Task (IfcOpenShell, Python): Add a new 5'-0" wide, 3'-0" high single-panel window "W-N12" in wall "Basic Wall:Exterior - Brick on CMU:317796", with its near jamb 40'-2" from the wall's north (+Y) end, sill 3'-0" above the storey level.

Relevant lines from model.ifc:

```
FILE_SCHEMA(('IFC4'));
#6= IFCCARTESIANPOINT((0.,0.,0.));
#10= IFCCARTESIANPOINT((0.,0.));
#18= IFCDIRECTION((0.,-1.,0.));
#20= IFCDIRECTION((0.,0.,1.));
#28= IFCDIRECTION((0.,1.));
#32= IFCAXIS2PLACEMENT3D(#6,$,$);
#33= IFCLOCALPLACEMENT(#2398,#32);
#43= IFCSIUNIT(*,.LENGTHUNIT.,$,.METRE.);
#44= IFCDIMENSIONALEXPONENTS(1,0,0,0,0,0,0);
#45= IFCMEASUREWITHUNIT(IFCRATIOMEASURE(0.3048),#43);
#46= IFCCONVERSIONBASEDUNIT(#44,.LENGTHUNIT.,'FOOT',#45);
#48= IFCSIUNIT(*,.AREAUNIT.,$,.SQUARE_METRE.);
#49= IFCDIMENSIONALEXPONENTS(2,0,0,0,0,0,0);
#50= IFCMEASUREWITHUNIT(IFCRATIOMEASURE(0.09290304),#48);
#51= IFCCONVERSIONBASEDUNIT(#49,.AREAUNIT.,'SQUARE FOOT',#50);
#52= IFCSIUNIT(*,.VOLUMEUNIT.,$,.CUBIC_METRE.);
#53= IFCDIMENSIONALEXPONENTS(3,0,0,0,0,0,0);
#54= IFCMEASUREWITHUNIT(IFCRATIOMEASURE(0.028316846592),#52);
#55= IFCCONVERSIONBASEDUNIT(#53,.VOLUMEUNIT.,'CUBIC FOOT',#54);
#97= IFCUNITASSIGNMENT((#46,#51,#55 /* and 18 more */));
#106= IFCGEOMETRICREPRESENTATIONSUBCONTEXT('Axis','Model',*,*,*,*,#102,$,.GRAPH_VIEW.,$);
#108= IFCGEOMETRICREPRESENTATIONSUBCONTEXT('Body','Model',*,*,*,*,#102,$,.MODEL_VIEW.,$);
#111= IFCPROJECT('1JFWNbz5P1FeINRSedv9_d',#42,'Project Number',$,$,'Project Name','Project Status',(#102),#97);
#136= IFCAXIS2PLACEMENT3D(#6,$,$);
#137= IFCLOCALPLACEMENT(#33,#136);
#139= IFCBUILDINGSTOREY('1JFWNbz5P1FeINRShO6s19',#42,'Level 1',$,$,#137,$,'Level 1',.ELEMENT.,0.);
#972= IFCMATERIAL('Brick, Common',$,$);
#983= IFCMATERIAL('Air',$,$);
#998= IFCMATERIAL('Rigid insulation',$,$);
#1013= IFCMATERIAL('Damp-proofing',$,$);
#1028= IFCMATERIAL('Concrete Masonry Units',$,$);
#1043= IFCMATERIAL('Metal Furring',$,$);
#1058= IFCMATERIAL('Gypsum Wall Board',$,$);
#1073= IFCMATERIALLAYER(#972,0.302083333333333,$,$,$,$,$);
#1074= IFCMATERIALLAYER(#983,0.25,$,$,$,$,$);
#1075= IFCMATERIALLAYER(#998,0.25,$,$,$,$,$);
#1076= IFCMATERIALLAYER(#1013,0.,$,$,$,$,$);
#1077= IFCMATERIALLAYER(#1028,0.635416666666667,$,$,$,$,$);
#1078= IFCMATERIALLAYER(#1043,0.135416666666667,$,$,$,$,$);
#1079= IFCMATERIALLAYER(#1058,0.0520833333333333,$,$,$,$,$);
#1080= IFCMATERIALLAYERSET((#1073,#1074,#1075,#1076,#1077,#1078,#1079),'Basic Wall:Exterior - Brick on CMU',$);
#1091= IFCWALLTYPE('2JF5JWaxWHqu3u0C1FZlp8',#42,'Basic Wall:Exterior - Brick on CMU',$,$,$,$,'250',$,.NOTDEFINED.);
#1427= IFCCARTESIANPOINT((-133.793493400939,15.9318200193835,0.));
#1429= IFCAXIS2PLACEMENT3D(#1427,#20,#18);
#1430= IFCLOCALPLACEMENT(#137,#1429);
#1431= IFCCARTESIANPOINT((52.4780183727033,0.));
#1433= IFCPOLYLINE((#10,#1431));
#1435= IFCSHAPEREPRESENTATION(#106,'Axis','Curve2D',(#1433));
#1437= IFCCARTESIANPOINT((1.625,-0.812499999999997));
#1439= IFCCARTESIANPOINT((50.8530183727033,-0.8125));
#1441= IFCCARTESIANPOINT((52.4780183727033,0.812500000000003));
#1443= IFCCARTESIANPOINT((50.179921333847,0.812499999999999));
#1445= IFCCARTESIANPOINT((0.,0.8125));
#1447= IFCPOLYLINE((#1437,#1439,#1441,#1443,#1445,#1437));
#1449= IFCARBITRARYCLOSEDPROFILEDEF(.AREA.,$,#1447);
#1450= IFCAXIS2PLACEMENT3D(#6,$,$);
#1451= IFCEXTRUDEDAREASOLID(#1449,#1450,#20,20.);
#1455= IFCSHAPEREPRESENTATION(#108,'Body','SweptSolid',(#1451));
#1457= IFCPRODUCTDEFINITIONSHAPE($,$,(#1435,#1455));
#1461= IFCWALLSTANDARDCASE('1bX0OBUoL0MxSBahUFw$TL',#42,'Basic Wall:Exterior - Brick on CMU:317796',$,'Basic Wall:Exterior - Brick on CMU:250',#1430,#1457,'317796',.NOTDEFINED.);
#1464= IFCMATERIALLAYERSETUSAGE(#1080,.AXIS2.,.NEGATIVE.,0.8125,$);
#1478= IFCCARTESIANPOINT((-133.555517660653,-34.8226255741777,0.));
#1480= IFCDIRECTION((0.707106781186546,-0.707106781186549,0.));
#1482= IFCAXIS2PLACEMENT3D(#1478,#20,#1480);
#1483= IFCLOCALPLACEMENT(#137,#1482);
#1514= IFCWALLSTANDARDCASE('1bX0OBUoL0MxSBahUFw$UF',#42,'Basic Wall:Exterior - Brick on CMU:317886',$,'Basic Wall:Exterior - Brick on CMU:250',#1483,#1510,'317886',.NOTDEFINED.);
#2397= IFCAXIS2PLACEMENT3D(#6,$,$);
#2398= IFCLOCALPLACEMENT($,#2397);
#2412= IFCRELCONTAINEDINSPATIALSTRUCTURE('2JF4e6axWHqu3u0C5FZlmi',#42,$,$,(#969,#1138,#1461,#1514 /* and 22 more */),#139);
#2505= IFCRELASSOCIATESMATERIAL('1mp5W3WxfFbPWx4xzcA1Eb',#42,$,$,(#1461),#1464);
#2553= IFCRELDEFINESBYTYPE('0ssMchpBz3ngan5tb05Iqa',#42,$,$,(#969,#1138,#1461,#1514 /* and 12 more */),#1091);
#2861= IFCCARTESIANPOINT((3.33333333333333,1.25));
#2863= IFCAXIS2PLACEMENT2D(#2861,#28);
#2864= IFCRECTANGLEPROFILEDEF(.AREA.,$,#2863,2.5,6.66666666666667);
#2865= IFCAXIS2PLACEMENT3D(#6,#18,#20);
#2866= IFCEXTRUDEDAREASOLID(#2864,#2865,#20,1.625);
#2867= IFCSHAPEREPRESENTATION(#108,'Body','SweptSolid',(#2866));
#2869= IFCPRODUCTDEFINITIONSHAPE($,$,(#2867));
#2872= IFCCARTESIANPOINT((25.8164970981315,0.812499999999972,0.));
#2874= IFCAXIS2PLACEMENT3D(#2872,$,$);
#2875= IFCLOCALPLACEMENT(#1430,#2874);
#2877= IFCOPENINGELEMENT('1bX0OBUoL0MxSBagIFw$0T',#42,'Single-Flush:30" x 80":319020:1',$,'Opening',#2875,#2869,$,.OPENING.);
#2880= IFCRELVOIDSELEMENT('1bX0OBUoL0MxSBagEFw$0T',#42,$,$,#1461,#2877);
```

```python
import numpy as np
import ifcopenshell
import ifcopenshell.api.feature
import ifcopenshell.api.geometry
import ifcopenshell.api.root
import ifcopenshell.api.spatial
import ifcopenshell.geom
import ifcopenshell.util.element
import ifcopenshell.util.placement
import ifcopenshell.util.representation
import ifcopenshell.util.shape
import ifcopenshell.util.unit

model = ifcopenshell.open("model.ifc")
unit_scale = ifcopenshell.util.unit.calculate_unit_scale(model)
settings = ifcopenshell.geom.settings()


def volume(element):
    """Net volume in cubic metres, openings subtracted."""
    shape = ifcopenshell.geom.create_shape(settings, element)
    return ifcopenshell.util.shape.get_volume(shape.geometry)


wall = model.by_guid("1bX0OBUoL0MxSBahUFw$TL")
storey = ifcopenshell.util.element.get_container(wall, ifc_class="IfcBuildingStorey")
context = ifcopenshell.util.representation.get_context(model, "Model", "Body", "MODEL_VIEW")
before = volume(wall)

width, height, from_end, sill = 1.524, 0.9144, 12.2428, 0.9144  # metres

# The wall runs along its own X axis, and the end named is its -X end.
wall_shape = ifcopenshell.geom.create_shape(settings, wall)
x, y, z = ifcopenshell.util.shape.get_vertices(wall_shape.geometry).T
start = x.min() + from_end
face, thickness = float(y.min()), float(y.max() - y.min())
wall_matrix = ifcopenshell.util.placement.get_local_placement(wall.ObjectPlacement)
level = ifcopenshell.util.placement.get_local_placement(storey.ObjectPlacement)[2, 3]


def in_wall(x, y):
    """Placement at x, y metres in the wall's axes, at sill height."""
    matrix = wall_matrix.copy()
    matrix[:, 3] = wall_matrix @ np.array([x / unit_scale, y / unit_scale, 0.0, 1.0])
    matrix[2, 3] = level + sill / unit_scale
    return matrix


# Opening: a box that overshoots both wall faces by 50 mm.
opening = ifcopenshell.api.root.create_entity(model, ifc_class="IfcOpeningElement", predefined_type="OPENING")
box = ifcopenshell.api.geometry.add_wall_representation(
    model, context=context, length=width, height=height, thickness=thickness + 0.1
)
ifcopenshell.api.geometry.assign_representation(model, product=opening, representation=box)
ifcopenshell.api.geometry.edit_object_placement(model, product=opening, matrix=in_wall(start, face - 0.05), is_si=False)
ifcopenshell.api.feature.add_feature(model, feature=opening, element=wall)

window = ifcopenshell.api.root.create_entity(model, ifc_class="IfcWindow", name="W-N12", predefined_type="WINDOW")
window.OverallWidth, window.OverallHeight = width / unit_scale, height / unit_scale
window.PartitioningType = "SINGLE_PANEL"
body = ifcopenshell.api.geometry.add_window_representation(
    model,
    context=context,
    overall_width=window.OverallWidth,
    overall_height=window.OverallHeight,
    partition_type="SINGLE_PANEL",
)
ifcopenshell.api.geometry.assign_representation(model, product=window, representation=body)
ifcopenshell.api.spatial.assign_container(model, products=[window], relating_structure=storey)
ifcopenshell.api.feature.add_filling(model, opening=opening, element=window)

# Centre the window in the wall's thickness.
ifcopenshell.api.geometry.edit_object_placement(model, product=window, matrix=in_wall(start, face), is_si=False)
window_shape = ifcopenshell.geom.create_shape(settings, window)
depth = ifcopenshell.util.shape.get_vertices(window_shape.geometry)[:, 1]
offset = face + thickness / 2 - (depth.min() + depth.max()) / 2
ifcopenshell.api.geometry.edit_object_placement(model, product=window, matrix=in_wall(start, offset), is_si=False)

after = volume(wall)

print(f"wall volume {before:.3f} -> {after:.3f} m3")

model.write("model_v2.ifc")
```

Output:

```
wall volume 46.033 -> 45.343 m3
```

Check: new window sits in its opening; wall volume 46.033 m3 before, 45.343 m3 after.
